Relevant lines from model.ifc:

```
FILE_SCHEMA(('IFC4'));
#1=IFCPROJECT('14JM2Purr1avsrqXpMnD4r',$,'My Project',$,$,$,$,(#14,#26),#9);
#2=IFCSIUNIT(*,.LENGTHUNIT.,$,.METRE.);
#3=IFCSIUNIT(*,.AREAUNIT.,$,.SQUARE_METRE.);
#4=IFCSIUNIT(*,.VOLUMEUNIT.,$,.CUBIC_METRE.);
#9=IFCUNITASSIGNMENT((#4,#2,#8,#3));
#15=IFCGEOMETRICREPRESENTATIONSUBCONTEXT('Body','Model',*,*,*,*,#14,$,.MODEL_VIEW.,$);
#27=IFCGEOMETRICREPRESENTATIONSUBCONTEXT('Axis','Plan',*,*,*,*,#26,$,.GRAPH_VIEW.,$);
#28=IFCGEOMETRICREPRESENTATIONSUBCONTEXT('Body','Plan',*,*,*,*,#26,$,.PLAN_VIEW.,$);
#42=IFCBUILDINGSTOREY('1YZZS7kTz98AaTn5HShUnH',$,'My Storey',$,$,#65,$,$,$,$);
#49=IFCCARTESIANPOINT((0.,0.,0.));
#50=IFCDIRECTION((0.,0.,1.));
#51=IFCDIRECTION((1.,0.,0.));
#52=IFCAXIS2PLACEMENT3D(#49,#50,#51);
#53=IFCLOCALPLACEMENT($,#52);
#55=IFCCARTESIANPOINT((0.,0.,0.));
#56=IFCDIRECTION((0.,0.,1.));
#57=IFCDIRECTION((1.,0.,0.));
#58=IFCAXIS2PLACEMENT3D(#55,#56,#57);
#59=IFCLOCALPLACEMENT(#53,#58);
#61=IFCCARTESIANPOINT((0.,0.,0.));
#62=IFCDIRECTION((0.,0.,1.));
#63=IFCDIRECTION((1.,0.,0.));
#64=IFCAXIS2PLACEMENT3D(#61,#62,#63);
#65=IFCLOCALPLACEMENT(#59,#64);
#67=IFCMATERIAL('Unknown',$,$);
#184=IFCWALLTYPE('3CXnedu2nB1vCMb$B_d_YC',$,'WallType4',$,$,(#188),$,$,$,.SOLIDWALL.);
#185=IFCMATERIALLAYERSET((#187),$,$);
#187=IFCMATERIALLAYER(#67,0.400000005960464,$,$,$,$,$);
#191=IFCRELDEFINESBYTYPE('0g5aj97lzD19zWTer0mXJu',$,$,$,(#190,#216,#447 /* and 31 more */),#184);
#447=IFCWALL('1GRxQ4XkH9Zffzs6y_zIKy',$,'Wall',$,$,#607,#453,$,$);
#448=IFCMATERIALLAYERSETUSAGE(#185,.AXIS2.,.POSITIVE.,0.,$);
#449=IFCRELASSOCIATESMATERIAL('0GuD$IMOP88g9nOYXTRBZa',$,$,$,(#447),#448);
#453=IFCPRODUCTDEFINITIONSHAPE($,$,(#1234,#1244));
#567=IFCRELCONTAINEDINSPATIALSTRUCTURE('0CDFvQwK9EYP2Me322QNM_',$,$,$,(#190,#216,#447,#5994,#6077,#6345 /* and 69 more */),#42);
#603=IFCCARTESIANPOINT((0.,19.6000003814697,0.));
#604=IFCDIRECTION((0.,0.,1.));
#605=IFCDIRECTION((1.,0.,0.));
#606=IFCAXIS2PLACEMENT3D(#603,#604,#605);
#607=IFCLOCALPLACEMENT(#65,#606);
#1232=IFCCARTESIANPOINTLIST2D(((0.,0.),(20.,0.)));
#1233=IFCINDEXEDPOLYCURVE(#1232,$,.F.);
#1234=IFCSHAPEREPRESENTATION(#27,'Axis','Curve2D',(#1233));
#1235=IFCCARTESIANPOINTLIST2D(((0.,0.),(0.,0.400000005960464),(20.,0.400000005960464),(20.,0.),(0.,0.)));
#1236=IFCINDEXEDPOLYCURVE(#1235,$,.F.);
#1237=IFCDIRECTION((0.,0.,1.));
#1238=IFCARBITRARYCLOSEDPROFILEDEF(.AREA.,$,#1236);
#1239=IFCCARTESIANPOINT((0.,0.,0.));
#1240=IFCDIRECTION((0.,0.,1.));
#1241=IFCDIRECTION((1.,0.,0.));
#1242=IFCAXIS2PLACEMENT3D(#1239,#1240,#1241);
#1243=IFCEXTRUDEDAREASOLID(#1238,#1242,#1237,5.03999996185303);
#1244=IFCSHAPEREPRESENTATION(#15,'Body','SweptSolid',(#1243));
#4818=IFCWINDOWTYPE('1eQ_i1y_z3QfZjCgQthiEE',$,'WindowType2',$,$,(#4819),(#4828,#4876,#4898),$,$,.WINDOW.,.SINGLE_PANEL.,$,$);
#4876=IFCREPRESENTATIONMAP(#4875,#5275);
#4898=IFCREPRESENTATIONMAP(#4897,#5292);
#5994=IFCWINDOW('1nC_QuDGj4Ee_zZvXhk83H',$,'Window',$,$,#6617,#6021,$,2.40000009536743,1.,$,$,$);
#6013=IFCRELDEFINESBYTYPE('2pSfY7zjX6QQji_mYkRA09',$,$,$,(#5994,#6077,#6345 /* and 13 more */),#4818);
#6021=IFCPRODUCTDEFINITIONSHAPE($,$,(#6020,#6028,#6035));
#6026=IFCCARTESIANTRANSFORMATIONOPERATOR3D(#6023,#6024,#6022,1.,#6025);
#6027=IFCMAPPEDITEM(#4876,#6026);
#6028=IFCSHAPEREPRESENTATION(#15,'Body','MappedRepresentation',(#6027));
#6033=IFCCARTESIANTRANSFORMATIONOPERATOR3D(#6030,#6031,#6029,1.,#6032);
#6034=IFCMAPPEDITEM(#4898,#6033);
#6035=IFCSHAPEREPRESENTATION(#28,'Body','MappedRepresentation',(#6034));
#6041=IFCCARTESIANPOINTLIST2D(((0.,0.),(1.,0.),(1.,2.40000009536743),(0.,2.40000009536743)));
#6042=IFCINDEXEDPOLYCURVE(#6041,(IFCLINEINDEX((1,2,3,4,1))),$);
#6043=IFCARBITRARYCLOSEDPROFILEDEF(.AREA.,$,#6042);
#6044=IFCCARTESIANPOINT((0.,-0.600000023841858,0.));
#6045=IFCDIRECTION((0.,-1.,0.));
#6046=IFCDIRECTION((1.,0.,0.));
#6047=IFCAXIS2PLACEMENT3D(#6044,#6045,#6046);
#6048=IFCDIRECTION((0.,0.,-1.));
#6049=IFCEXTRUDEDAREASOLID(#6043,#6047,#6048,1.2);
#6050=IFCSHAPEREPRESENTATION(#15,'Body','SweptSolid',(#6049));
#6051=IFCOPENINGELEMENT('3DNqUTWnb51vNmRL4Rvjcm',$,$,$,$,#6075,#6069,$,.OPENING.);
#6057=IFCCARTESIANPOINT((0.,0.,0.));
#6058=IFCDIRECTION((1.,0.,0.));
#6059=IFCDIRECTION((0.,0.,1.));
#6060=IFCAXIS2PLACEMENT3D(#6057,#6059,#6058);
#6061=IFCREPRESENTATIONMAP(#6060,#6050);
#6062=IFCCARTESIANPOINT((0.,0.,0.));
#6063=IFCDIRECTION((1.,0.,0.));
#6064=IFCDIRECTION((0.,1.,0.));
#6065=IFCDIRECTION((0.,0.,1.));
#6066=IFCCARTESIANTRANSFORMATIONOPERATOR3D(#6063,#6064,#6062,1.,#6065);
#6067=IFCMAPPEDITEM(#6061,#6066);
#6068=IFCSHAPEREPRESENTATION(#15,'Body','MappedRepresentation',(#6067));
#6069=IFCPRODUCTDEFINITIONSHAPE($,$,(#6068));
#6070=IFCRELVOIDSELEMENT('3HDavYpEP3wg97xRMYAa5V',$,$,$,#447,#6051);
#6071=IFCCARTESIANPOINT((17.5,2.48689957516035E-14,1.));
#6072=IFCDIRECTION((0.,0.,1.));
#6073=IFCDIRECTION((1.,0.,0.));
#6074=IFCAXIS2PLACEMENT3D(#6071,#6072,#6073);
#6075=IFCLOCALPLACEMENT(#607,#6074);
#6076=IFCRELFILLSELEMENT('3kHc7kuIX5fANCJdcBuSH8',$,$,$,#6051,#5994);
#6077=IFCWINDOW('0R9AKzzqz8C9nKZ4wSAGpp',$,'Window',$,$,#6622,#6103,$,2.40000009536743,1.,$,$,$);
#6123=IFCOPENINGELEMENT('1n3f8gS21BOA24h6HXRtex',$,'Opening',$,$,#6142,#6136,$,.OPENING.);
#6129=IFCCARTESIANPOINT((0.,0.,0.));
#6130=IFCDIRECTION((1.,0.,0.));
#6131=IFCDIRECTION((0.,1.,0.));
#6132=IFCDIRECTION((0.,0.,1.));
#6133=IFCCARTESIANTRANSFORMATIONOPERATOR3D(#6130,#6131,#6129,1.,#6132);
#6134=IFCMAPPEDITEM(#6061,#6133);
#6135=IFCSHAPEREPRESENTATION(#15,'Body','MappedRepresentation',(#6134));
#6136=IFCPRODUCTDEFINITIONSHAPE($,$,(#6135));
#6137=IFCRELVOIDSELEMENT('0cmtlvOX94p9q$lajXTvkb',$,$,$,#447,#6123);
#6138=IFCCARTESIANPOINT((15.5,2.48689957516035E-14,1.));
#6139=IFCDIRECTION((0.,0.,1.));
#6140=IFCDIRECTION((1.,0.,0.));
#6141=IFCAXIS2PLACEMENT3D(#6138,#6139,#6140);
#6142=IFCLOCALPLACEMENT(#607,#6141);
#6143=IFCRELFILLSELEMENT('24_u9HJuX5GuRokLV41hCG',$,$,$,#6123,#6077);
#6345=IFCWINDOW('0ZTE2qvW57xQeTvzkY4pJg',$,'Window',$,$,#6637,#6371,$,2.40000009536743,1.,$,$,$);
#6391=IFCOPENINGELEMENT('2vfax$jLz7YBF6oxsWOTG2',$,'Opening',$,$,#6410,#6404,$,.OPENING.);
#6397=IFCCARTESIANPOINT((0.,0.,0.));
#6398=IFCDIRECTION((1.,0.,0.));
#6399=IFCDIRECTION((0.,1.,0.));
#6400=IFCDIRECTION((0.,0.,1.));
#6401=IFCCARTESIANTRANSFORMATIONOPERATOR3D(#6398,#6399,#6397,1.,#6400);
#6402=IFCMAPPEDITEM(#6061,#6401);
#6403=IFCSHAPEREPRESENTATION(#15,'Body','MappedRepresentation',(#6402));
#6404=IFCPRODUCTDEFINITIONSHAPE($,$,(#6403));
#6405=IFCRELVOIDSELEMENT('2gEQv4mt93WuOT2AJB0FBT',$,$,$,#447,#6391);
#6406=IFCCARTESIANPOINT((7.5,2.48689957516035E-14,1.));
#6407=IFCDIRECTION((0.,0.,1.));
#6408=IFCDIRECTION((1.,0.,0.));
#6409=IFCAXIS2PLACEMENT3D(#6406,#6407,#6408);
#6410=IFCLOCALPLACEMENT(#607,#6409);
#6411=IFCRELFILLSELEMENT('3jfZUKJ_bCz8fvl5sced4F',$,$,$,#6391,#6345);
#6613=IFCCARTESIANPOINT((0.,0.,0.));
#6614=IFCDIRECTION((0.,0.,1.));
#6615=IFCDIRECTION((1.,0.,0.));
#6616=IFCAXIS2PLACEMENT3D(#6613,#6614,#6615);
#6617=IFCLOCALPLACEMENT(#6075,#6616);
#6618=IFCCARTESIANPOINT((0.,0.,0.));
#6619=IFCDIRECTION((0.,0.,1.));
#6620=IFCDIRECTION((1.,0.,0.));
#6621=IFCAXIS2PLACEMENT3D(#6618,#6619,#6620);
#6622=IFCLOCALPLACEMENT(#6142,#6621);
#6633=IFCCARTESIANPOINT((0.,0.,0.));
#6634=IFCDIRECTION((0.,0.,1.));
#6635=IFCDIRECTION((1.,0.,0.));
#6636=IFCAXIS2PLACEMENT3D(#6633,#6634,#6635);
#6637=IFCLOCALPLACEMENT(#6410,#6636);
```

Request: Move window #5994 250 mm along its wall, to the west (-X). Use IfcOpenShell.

```python
import ifcopenshell
import ifcopenshell.api.geometry
import ifcopenshell.util.placement

model = ifcopenshell.open("model.ifc")

window = model.by_id(5994)
opening = window.FillsVoids[0].RelatingOpeningElement
wall = opening.VoidsElements[0].RelatingBuildingElement

wall_matrix = ifcopenshell.util.placement.get_local_placement(wall.ObjectPlacement)
shift = wall_matrix[:3, 0] * -0.25
before = ifcopenshell.util.placement.get_local_placement(window.ObjectPlacement)[:3, 3].copy()

# The window is placed relative to its opening, so it follows when the opening moves.
matrix = ifcopenshell.util.placement.get_local_placement(opening.ObjectPlacement)
matrix[:3, 3] += shift
ifcopenshell.api.geometry.edit_object_placement(
    model, product=opening, matrix=matrix, is_si=False, should_transform_children=True
)

after = ifcopenshell.util.placement.get_local_placement(window.ObjectPlacement)[:3, 3]
print("window moved by", (after - before).round(3) + 0.0)

model.write("model_edited.ifc")
```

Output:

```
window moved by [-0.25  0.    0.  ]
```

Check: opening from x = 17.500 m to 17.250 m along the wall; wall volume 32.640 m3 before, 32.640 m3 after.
